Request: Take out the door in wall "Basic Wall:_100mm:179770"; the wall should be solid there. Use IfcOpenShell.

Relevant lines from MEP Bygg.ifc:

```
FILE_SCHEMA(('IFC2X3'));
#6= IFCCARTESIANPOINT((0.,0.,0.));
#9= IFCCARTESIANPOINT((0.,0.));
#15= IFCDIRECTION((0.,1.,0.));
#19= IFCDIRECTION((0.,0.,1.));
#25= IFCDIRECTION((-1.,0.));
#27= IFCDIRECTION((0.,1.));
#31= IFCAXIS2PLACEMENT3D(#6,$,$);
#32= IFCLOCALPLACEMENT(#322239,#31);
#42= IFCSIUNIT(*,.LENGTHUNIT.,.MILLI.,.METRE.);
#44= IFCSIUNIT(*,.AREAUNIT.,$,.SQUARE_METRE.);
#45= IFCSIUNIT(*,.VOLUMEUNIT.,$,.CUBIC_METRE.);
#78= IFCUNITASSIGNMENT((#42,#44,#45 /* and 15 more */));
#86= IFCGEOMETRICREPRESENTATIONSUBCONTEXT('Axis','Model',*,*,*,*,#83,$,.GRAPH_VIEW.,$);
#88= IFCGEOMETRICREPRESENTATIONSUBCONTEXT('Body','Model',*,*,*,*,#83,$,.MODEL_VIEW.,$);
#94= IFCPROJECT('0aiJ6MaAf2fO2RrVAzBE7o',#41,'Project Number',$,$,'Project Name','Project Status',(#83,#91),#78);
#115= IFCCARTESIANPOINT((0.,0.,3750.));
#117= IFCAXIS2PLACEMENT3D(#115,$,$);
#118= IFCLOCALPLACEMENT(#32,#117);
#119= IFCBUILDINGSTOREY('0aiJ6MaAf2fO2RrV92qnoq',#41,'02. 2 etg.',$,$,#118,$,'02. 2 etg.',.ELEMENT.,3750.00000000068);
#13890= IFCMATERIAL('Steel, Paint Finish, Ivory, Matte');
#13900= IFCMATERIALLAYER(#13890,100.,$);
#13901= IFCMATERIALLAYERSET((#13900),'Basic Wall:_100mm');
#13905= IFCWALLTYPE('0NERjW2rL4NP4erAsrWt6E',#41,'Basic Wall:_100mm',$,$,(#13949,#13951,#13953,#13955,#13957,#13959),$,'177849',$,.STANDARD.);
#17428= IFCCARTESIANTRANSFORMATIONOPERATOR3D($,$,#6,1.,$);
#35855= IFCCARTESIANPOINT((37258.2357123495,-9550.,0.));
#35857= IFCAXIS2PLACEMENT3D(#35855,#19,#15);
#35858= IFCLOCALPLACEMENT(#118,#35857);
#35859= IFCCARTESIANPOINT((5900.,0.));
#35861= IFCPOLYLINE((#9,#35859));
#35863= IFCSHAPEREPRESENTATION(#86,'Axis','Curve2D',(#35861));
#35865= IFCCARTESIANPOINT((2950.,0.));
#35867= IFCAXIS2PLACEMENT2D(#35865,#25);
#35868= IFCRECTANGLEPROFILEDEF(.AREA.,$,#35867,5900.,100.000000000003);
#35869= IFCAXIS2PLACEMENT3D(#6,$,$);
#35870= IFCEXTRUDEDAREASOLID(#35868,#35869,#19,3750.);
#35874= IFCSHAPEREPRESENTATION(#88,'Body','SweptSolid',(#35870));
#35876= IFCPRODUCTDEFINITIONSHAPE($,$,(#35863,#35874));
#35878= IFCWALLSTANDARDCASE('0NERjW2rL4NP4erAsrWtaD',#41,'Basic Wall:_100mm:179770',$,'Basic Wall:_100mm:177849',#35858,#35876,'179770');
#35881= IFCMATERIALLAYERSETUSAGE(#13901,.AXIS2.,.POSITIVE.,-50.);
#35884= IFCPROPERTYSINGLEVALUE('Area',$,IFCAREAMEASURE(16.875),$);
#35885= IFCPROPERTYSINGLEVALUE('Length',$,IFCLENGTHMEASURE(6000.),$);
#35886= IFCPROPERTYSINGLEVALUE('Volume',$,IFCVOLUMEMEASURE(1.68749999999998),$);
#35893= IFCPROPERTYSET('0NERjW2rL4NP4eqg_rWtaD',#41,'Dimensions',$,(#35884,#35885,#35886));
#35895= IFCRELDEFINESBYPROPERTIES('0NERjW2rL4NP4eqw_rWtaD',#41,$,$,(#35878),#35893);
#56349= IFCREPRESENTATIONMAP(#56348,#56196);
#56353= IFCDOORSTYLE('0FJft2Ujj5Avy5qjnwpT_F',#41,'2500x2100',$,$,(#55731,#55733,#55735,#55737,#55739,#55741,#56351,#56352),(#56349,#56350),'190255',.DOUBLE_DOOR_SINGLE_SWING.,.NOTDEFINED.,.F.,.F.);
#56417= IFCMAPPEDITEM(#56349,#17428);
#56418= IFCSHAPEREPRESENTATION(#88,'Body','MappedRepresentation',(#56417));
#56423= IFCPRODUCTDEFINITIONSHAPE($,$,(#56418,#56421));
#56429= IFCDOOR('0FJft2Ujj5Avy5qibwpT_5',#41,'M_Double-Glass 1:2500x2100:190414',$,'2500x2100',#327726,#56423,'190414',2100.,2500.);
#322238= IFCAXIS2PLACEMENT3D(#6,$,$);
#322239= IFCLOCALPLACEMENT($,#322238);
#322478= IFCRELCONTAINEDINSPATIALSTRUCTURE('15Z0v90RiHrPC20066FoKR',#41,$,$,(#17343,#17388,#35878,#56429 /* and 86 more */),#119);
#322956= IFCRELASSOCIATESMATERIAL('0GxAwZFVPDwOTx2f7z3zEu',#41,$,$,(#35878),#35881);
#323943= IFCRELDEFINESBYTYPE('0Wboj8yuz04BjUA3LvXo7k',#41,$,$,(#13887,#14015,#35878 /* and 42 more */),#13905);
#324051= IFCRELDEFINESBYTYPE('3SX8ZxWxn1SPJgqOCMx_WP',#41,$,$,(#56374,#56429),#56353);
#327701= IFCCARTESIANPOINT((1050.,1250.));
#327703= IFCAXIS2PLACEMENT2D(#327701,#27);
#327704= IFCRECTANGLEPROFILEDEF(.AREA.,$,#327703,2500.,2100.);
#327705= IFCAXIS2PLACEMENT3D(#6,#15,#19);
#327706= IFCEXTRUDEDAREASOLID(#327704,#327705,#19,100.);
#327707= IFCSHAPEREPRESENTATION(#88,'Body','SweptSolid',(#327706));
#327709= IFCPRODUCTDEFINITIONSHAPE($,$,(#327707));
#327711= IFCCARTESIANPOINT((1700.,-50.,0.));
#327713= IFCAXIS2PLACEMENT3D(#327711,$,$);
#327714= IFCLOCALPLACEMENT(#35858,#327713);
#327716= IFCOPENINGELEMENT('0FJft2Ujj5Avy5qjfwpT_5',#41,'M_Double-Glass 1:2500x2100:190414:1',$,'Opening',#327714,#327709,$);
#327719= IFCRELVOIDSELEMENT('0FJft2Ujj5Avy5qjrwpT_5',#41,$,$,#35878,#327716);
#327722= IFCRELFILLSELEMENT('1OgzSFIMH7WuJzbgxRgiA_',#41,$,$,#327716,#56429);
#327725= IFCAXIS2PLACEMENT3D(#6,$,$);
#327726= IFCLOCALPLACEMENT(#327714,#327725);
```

```python
import ifcopenshell
import ifcopenshell.api.feature
import ifcopenshell.api.pset
import ifcopenshell.api.root
import ifcopenshell.geom
import ifcopenshell.util.element
import ifcopenshell.util.shape
import ifcopenshell.util.unit

model = ifcopenshell.open("MEP Bygg.ifc")
area_scale = ifcopenshell.util.unit.calculate_unit_scale(model, "AREAUNIT")
volume_scale = ifcopenshell.util.unit.calculate_unit_scale(model, "VOLUMEUNIT")
settings = ifcopenshell.geom.settings()


def volume(element):
    """Net volume in cubic metres, openings subtracted."""
    shape = ifcopenshell.geom.create_shape(settings, element)
    return ifcopenshell.util.shape.get_volume(shape.geometry)


door = model.by_id(56429)
opening = door.FillsVoids[0].RelatingOpeningElement
wall = opening.VoidsElements[0].RelatingBuildingElement
before = volume(wall)

ifcopenshell.api.root.remove_product(model, product=door)
ifcopenshell.api.feature.remove_feature(model, feature=opening)

after = volume(wall)
thickness = 0.1  # wall thickness in metres

# Update the wall's stored quantities.
pset = model.by_id(ifcopenshell.util.element.get_pset(wall, "Dimensions", should_inherit=False)["id"])
ifcopenshell.api.pset.edit_pset(model, pset=pset, properties={
    "Area": model.create_entity("IfcAreaMeasure", after / thickness / area_scale),
    "Volume": model.create_entity("IfcVolumeMeasure", after / volume_scale),
})

print(f"wall volume {before:.3f} -> {after:.3f} m3")

model.write("MEP Bygg_rev.ifc")
```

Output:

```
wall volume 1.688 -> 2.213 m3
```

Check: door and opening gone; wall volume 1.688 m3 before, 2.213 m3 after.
